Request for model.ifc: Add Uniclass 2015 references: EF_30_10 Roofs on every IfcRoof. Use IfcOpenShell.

First a look at what the model holds.

```python
import ifcopenshell

model = ifcopenshell.open("model.ifc")
print(model.schema)
print("classifications:", [c.Name for c in model.by_type("IfcClassification")])
for ifc_class in ("IfcDoor", "IfcRoof", "IfcStair", "IfcWall", "IfcWindow"):
    print(ifc_class, len(model.by_type(ifc_class)))
```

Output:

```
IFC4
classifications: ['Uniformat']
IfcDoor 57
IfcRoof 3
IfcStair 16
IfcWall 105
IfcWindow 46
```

```python
import ifcopenshell
import ifcopenshell.api.classification

model = ifcopenshell.open("model.ifc")

system = ifcopenshell.api.classification.add_classification(model, classification="Uniclass 2015")

codes = {
    "IfcRoof": ("EF_30_10", "Roofs"),
}
for ifc_class, (code, name) in codes.items():
    products = model.by_type(ifc_class)
    ifcopenshell.api.classification.add_reference(
        model, products=products, classification=system, identification=code, name=name
    )
    print(code, len(products))

model.write("model_rev.ifc")
```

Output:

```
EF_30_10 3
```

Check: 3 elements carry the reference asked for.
